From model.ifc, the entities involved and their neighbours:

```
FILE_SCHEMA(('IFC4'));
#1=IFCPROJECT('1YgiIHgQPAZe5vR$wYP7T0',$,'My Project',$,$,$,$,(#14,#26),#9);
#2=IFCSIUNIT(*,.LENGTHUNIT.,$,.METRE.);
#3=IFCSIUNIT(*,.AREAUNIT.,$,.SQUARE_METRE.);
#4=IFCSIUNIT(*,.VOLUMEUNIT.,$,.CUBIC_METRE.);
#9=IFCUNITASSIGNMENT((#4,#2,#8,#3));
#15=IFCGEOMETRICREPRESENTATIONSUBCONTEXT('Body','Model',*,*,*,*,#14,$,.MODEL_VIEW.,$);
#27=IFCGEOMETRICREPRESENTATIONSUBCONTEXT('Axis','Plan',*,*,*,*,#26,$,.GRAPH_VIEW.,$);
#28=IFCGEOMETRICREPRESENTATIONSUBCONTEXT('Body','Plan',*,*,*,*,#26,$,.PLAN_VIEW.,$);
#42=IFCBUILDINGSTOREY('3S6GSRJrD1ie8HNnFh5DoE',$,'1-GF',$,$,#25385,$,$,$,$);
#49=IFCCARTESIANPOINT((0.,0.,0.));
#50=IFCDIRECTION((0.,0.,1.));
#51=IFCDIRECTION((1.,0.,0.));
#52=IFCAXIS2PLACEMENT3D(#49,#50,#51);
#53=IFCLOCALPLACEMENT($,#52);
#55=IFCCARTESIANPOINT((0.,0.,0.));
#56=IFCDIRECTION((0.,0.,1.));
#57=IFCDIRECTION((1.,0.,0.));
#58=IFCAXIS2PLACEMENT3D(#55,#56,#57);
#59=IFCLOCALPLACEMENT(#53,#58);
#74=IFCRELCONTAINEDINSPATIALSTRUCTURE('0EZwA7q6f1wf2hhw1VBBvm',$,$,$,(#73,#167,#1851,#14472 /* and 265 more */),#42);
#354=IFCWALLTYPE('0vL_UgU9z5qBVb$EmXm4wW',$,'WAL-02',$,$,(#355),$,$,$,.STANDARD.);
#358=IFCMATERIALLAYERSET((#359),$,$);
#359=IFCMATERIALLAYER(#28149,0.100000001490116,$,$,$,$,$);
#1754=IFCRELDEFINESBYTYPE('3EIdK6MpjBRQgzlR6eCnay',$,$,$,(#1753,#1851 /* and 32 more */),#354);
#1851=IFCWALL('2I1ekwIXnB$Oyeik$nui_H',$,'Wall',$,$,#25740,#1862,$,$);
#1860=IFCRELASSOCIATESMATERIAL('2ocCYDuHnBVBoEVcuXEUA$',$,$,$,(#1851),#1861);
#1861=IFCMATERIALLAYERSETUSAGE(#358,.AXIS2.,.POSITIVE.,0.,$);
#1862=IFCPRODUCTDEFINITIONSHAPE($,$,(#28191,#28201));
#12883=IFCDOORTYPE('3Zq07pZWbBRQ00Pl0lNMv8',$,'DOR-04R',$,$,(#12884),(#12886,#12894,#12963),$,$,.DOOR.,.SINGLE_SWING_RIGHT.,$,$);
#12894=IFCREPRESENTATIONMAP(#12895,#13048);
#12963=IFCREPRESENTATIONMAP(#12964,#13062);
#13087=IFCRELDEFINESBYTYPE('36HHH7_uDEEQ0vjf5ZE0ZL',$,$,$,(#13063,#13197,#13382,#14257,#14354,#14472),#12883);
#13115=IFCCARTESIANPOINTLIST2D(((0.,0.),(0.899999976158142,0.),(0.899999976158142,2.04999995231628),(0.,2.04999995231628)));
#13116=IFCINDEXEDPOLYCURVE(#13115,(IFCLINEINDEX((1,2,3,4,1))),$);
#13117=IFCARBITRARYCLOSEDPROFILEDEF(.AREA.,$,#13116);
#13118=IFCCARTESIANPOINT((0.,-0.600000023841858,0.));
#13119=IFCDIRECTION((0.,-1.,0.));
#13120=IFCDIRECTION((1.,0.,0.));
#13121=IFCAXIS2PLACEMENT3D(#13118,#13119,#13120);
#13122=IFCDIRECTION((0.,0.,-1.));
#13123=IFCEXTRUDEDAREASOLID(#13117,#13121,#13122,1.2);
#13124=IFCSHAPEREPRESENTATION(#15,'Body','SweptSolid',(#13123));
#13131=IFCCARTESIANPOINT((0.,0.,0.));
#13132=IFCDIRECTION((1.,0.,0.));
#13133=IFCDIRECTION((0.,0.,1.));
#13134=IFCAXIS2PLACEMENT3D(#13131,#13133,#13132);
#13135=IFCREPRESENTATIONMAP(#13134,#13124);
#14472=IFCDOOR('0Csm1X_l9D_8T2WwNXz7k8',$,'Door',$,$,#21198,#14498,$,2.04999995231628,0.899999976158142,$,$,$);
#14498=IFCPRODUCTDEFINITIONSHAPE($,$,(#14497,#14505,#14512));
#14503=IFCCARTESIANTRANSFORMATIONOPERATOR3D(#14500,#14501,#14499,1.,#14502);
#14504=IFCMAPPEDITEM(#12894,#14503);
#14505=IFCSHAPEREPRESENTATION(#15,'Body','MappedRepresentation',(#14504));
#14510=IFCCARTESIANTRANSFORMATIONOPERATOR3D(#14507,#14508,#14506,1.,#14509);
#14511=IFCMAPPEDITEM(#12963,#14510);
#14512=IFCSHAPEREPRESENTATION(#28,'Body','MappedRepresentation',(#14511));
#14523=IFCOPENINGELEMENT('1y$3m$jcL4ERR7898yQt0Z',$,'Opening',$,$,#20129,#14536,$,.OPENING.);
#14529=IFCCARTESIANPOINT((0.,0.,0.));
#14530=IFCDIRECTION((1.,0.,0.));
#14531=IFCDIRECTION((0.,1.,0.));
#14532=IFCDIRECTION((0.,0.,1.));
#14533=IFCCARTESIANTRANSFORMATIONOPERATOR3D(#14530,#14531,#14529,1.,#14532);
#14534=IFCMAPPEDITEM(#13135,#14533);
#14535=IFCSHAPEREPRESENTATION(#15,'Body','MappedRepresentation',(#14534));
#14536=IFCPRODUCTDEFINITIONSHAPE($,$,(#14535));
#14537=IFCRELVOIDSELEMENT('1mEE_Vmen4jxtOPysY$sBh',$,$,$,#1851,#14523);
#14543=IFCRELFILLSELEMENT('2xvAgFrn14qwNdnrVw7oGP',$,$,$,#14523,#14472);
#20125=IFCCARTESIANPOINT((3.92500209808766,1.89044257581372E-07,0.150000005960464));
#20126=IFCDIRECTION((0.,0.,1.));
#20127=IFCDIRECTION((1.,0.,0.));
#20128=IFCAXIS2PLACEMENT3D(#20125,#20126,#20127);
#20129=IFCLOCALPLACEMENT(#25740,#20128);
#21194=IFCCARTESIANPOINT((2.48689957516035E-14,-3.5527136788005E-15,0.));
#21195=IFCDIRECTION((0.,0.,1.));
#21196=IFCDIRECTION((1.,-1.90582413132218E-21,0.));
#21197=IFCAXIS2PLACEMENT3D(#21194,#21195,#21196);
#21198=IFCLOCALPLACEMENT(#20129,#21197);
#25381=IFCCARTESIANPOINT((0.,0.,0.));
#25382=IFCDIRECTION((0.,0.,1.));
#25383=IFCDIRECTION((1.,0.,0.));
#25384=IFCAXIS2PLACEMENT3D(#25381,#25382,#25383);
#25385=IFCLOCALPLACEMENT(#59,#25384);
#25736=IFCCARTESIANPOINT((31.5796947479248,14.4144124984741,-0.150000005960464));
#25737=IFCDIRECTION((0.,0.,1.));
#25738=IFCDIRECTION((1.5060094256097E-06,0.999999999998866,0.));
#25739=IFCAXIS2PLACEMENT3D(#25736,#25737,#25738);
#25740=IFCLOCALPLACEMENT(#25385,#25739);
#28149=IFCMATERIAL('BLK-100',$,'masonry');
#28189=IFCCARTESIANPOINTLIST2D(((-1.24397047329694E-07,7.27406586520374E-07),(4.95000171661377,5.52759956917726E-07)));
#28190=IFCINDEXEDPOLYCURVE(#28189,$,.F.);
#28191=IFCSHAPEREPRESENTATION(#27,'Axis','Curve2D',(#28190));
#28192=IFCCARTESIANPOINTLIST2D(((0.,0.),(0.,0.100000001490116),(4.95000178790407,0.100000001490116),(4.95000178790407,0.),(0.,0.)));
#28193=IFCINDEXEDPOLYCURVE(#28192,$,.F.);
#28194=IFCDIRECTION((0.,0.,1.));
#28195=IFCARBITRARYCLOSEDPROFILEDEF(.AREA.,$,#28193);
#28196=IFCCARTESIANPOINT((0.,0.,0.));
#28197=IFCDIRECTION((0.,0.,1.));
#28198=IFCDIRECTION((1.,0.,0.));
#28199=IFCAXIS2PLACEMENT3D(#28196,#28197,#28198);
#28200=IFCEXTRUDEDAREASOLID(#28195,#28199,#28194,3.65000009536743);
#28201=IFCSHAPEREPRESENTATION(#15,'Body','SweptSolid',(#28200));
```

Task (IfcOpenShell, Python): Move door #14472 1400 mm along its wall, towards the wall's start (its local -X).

```python
import ifcopenshell
import ifcopenshell.api.geometry
import ifcopenshell.util.placement

model = ifcopenshell.open("model.ifc")

door = model.by_guid("0Csm1X_l9D_8T2WwNXz7k8")
opening = door.FillsVoids[0].RelatingOpeningElement
wall = opening.VoidsElements[0].RelatingBuildingElement

wall_matrix = ifcopenshell.util.placement.get_local_placement(wall.ObjectPlacement)
shift = wall_matrix[:3, 0] * -1.4
before = ifcopenshell.util.placement.get_local_placement(door.ObjectPlacement)[:3, 3].copy()

# The door is placed relative to its opening, so it follows when the opening moves.
matrix = ifcopenshell.util.placement.get_local_placement(opening.ObjectPlacement)
matrix[:3, 3] += shift
ifcopenshell.api.geometry.edit_object_placement(
    model, product=opening, matrix=matrix, is_si=False, should_transform_children=True
)

after = ifcopenshell.util.placement.get_local_placement(door.ObjectPlacement)[:3, 3]
print("door moved by", (after - before).round(3) + 0.0)

model.write("model_updated.ifc")
```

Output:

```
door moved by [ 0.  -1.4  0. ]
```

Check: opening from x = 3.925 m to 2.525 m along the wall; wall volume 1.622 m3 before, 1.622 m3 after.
